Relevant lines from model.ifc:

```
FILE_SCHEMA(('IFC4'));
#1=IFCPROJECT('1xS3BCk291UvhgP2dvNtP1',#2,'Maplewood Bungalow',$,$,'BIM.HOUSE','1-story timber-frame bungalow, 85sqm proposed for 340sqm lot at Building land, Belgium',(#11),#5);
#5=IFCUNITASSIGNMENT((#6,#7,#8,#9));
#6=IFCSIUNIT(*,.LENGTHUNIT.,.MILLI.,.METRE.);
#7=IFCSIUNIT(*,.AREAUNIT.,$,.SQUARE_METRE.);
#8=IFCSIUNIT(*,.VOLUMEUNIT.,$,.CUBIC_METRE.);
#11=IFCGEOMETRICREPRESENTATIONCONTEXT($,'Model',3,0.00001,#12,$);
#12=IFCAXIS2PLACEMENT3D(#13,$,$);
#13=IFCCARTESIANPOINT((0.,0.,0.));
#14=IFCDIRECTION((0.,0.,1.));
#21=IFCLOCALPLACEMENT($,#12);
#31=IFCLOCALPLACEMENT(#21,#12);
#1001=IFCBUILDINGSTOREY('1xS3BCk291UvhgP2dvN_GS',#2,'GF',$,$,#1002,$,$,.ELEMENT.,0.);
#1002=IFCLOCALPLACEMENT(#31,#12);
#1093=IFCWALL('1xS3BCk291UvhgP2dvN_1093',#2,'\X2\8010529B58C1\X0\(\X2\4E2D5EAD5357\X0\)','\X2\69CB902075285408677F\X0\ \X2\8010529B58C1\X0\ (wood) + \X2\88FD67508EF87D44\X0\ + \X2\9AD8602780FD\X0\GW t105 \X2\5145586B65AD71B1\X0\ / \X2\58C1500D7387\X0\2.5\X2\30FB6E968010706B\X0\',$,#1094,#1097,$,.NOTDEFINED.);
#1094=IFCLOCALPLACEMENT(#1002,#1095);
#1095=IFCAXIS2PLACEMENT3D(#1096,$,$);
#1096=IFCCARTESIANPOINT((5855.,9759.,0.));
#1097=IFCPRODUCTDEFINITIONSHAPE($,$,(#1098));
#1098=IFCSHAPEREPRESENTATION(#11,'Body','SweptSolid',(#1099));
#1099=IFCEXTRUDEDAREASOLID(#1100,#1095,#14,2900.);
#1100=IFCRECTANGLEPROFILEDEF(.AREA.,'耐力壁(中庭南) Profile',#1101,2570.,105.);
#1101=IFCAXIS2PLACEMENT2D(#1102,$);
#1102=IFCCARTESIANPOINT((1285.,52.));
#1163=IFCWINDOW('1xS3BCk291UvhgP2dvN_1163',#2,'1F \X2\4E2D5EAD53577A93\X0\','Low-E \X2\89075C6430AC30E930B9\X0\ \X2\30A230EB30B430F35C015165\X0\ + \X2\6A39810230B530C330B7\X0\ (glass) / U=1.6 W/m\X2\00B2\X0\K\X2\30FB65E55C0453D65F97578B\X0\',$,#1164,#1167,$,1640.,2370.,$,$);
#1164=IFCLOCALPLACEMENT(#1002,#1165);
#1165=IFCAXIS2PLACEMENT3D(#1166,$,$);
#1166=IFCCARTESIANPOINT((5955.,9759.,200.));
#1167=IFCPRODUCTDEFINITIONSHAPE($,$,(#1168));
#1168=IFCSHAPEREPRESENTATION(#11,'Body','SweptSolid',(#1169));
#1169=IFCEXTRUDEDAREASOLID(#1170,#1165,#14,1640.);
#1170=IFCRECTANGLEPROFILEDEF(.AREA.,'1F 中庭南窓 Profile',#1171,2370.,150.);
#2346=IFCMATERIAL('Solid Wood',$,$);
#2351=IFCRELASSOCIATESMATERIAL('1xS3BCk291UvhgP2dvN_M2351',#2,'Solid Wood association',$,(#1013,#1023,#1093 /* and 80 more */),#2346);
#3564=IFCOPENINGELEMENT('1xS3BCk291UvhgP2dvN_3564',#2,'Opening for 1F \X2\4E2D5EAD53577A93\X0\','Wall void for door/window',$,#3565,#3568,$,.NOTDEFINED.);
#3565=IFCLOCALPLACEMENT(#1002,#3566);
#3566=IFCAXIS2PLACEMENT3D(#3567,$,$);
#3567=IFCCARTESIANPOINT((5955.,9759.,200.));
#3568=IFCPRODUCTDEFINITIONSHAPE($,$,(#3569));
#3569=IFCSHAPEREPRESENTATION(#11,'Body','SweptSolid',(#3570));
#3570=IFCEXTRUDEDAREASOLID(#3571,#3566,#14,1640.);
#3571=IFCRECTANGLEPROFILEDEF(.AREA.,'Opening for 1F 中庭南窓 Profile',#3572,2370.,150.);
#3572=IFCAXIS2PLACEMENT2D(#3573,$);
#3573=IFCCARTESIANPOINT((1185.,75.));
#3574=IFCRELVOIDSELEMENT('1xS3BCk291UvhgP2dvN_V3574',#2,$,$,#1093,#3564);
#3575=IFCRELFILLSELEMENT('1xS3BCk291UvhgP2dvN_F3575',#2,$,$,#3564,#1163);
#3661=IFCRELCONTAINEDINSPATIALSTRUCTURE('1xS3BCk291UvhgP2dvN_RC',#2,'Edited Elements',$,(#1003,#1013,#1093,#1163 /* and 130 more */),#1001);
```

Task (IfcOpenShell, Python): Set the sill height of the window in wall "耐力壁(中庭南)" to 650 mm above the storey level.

```python
import numpy as np
import ifcopenshell
import ifcopenshell.api.geometry
import ifcopenshell.geom
import ifcopenshell.util.element
import ifcopenshell.util.placement
import ifcopenshell.util.shape
import ifcopenshell.util.unit

model = ifcopenshell.open("model.ifc")
unit_scale = ifcopenshell.util.unit.calculate_unit_scale(model)

window = model.by_guid("1xS3BCk291UvhgP2dvN_1163")
opening = window.FillsVoids[0].RelatingOpeningElement
storey = ifcopenshell.util.element.get_container(window, ifc_class="IfcBuildingStorey")
level = ifcopenshell.util.placement.get_local_placement(storey.ObjectPlacement)[2, 3]

# The opening's origin need not be at the sill, so measure its lowest point.
shape = ifcopenshell.geom.create_shape(ifcopenshell.geom.settings(), opening)
bottom = ifcopenshell.util.shape.get_shape_bottom_elevation(shape, shape.geometry) / unit_scale
dz = level + 0.65 / unit_scale - bottom

shift = np.array([0.0, 0.0, dz])
# The window is not placed relative to its opening, so move both.
for product in (opening, window):
    matrix = ifcopenshell.util.placement.get_local_placement(product.ObjectPlacement)
    matrix[:3, 3] += shift
    ifcopenshell.api.geometry.edit_object_placement(model, product=product, matrix=matrix, is_si=False)

print(f"moved by {dz * unit_scale:+.3f} m")

model.write("model_edited.ifc")
```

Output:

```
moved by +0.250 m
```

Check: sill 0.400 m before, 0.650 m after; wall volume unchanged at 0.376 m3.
